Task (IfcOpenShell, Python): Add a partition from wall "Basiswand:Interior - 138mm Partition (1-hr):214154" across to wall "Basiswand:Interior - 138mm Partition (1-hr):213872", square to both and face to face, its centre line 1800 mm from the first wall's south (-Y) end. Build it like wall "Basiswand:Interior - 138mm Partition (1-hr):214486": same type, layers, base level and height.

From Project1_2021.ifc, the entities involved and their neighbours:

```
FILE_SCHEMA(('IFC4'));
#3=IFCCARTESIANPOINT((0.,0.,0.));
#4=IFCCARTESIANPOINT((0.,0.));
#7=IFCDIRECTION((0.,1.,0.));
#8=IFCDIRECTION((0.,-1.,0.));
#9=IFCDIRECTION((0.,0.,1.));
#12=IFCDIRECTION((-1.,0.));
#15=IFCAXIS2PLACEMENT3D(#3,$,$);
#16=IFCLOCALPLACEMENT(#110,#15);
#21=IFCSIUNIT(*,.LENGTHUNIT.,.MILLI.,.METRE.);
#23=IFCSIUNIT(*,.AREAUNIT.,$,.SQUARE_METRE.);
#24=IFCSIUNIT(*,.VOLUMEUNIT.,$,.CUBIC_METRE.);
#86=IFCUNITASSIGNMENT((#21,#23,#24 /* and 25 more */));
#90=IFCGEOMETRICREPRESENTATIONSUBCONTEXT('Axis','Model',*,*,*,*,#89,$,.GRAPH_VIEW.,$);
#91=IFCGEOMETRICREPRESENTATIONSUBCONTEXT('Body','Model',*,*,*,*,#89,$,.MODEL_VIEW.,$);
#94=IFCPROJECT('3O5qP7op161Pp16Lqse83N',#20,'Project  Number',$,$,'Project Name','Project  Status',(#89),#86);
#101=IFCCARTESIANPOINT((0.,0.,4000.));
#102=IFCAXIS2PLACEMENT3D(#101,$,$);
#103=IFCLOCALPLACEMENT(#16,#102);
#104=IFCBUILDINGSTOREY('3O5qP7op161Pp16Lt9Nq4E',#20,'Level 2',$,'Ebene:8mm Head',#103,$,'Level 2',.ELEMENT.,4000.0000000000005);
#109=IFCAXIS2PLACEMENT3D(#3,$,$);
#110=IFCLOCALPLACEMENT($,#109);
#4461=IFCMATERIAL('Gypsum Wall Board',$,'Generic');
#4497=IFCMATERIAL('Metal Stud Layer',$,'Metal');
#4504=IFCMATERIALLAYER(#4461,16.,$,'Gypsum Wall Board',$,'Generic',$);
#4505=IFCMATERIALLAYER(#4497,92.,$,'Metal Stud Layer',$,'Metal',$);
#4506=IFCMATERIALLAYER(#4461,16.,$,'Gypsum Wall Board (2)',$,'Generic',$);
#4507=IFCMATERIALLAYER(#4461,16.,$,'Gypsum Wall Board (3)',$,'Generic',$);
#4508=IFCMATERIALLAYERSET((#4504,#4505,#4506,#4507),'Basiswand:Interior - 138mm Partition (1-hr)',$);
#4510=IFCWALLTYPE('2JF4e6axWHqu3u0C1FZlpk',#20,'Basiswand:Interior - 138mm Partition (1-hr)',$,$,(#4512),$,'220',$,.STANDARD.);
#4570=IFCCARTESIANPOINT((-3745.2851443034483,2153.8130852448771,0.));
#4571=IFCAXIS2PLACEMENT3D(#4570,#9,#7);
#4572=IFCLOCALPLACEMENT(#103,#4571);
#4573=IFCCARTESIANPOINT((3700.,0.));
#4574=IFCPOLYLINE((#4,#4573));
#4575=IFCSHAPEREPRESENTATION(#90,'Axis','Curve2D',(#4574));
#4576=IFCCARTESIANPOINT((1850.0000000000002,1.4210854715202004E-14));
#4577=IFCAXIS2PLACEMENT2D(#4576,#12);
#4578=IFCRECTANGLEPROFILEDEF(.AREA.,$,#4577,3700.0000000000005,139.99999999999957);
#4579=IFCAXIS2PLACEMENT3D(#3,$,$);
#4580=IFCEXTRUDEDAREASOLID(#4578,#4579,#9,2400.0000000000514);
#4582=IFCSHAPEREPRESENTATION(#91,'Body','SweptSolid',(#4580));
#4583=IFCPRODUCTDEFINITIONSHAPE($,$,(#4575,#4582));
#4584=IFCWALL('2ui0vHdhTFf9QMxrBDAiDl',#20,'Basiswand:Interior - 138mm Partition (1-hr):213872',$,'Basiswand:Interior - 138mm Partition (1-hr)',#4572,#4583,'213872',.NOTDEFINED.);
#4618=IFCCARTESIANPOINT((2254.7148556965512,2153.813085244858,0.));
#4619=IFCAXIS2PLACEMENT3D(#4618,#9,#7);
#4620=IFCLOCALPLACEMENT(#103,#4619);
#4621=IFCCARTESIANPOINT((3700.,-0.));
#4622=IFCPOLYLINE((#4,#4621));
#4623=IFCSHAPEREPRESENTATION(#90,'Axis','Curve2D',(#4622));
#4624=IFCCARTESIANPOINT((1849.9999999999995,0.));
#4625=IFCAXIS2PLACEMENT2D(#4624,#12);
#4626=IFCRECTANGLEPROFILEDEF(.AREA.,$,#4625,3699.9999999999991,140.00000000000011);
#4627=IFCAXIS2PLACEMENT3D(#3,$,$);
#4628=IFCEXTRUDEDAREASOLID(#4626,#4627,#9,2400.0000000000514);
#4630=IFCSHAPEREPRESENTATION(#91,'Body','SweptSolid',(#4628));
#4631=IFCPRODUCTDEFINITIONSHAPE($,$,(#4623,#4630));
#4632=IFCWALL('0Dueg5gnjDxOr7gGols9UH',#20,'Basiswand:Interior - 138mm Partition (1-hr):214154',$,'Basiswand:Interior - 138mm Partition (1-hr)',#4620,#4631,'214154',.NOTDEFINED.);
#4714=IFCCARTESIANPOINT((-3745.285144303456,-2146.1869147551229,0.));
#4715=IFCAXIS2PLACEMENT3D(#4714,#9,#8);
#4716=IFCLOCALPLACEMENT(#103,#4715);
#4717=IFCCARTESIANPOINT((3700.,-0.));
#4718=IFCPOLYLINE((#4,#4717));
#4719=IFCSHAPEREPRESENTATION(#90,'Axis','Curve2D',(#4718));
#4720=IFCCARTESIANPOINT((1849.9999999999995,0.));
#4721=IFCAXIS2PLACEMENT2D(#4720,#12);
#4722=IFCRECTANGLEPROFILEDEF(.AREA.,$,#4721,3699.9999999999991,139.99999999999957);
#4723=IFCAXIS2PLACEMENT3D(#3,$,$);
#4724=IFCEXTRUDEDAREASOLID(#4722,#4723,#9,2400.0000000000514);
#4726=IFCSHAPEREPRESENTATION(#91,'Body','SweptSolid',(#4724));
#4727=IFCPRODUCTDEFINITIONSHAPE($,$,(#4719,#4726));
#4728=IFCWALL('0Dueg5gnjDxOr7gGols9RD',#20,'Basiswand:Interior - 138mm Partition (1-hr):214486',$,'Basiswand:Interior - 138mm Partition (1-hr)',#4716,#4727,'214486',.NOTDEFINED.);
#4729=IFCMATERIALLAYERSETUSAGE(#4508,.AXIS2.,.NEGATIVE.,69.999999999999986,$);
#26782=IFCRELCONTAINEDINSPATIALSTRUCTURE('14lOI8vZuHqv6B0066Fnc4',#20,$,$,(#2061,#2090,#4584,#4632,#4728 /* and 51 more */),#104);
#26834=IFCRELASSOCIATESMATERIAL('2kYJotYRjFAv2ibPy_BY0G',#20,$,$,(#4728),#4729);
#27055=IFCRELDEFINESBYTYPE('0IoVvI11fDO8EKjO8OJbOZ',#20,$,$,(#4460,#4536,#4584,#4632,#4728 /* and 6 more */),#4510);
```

```python
import numpy as np
import ifcopenshell
import ifcopenshell.api.geometry
import ifcopenshell.api.material
import ifcopenshell.api.pset
import ifcopenshell.api.root
import ifcopenshell.api.spatial
import ifcopenshell.api.type
import ifcopenshell.geom
import ifcopenshell.util.element
import ifcopenshell.util.placement
import ifcopenshell.util.representation
import ifcopenshell.util.shape
import ifcopenshell.util.unit

model = ifcopenshell.open("Project1_2021.ifc")
unit_scale = ifcopenshell.util.unit.calculate_unit_scale(model)
settings = ifcopenshell.geom.settings()
settings.set("use-world-coords", True)

start_wall = model.by_guid("0Dueg5gnjDxOr7gGols9UH")
end_wall = model.by_guid("2ui0vHdhTFf9QMxrBDAiDl")
like = model.by_guid("0Dueg5gnjDxOr7gGols9RD")
matrix = ifcopenshell.util.placement.get_local_placement(start_wall.ObjectPlacement)
matrix[:3, 3] *= unit_scale


def extent(element):
    """Bounding box in the first wall's axes, in metres."""
    shape = ifcopenshell.geom.create_shape(settings, element)
    points = (ifcopenshell.util.shape.get_vertices(shape.geometry) - matrix[:3, 3]) @ matrix[:3, :3]
    return points.min(axis=0), points.max(axis=0)


y_start = extent(start_wall)[1][1]
y_end = extent(end_wall)[0][1]
like_min, like_max = extent(like)
length, height = float(abs(y_end - y_start)), float(like_max[2] - like_min[2])
layer_set = ifcopenshell.util.element.get_material(like, should_skip_usage=True)
thickness = sum(layer.LayerThickness for layer in layer_set.MaterialLayers) * unit_scale

wall = ifcopenshell.api.root.create_entity(model, ifc_class="IfcWall", name="New partition")
storey = ifcopenshell.util.element.get_container(like)
ifcopenshell.api.spatial.assign_container(model, products=[wall], relating_structure=storey)
ifcopenshell.api.type.assign_type(
    model, related_objects=[wall], relating_type=ifcopenshell.util.element.get_type(like), should_map_representations=False
)
rel = ifcopenshell.api.material.assign_material(
    model, products=[wall], type="IfcMaterialLayerSetUsage", material=layer_set
)
rel.RelatingMaterial.OffsetFromReferenceLine = -thickness / 2 / unit_scale
pset = ifcopenshell.api.pset.add_pset(model, product=wall, name="Pset_WallCommon")
ifcopenshell.api.pset.edit_pset(model, pset=pset, properties={"IsExternal": False, "LoadBearing": False})

# The axis runs down the middle of the wall.
axis = ifcopenshell.api.geometry.add_axis_representation(
    model, context=ifcopenshell.util.representation.get_context(model, "Model", "Axis"), axis=[(0.0, 0.0), (length, 0.0)]
)
body = ifcopenshell.api.geometry.add_wall_representation(
    model,
    context=ifcopenshell.util.representation.get_context(model, "Model", "Body", "MODEL_VIEW"),
    length=length,
    height=height,
    thickness=thickness,
    offset=-thickness / 2,
)
for representation in (axis, body):
    ifcopenshell.api.geometry.assign_representation(model, product=wall, representation=representation)

placement = matrix @ ifcopenshell.util.placement.rotation(90, "Z")
placement[:, 3] = matrix @ np.array([extent(start_wall)[0][0] + 1.8, y_start, like_min[2], 1.0])
ifcopenshell.api.geometry.edit_object_placement(model, product=wall, matrix=placement)

print(f"partition {length:.3f} m long, {height:.3f} m high, {thickness:.3f} m thick")

model.write("Project1_2021-out.ifc")
```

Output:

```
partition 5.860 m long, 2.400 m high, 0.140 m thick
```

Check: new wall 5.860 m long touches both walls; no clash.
